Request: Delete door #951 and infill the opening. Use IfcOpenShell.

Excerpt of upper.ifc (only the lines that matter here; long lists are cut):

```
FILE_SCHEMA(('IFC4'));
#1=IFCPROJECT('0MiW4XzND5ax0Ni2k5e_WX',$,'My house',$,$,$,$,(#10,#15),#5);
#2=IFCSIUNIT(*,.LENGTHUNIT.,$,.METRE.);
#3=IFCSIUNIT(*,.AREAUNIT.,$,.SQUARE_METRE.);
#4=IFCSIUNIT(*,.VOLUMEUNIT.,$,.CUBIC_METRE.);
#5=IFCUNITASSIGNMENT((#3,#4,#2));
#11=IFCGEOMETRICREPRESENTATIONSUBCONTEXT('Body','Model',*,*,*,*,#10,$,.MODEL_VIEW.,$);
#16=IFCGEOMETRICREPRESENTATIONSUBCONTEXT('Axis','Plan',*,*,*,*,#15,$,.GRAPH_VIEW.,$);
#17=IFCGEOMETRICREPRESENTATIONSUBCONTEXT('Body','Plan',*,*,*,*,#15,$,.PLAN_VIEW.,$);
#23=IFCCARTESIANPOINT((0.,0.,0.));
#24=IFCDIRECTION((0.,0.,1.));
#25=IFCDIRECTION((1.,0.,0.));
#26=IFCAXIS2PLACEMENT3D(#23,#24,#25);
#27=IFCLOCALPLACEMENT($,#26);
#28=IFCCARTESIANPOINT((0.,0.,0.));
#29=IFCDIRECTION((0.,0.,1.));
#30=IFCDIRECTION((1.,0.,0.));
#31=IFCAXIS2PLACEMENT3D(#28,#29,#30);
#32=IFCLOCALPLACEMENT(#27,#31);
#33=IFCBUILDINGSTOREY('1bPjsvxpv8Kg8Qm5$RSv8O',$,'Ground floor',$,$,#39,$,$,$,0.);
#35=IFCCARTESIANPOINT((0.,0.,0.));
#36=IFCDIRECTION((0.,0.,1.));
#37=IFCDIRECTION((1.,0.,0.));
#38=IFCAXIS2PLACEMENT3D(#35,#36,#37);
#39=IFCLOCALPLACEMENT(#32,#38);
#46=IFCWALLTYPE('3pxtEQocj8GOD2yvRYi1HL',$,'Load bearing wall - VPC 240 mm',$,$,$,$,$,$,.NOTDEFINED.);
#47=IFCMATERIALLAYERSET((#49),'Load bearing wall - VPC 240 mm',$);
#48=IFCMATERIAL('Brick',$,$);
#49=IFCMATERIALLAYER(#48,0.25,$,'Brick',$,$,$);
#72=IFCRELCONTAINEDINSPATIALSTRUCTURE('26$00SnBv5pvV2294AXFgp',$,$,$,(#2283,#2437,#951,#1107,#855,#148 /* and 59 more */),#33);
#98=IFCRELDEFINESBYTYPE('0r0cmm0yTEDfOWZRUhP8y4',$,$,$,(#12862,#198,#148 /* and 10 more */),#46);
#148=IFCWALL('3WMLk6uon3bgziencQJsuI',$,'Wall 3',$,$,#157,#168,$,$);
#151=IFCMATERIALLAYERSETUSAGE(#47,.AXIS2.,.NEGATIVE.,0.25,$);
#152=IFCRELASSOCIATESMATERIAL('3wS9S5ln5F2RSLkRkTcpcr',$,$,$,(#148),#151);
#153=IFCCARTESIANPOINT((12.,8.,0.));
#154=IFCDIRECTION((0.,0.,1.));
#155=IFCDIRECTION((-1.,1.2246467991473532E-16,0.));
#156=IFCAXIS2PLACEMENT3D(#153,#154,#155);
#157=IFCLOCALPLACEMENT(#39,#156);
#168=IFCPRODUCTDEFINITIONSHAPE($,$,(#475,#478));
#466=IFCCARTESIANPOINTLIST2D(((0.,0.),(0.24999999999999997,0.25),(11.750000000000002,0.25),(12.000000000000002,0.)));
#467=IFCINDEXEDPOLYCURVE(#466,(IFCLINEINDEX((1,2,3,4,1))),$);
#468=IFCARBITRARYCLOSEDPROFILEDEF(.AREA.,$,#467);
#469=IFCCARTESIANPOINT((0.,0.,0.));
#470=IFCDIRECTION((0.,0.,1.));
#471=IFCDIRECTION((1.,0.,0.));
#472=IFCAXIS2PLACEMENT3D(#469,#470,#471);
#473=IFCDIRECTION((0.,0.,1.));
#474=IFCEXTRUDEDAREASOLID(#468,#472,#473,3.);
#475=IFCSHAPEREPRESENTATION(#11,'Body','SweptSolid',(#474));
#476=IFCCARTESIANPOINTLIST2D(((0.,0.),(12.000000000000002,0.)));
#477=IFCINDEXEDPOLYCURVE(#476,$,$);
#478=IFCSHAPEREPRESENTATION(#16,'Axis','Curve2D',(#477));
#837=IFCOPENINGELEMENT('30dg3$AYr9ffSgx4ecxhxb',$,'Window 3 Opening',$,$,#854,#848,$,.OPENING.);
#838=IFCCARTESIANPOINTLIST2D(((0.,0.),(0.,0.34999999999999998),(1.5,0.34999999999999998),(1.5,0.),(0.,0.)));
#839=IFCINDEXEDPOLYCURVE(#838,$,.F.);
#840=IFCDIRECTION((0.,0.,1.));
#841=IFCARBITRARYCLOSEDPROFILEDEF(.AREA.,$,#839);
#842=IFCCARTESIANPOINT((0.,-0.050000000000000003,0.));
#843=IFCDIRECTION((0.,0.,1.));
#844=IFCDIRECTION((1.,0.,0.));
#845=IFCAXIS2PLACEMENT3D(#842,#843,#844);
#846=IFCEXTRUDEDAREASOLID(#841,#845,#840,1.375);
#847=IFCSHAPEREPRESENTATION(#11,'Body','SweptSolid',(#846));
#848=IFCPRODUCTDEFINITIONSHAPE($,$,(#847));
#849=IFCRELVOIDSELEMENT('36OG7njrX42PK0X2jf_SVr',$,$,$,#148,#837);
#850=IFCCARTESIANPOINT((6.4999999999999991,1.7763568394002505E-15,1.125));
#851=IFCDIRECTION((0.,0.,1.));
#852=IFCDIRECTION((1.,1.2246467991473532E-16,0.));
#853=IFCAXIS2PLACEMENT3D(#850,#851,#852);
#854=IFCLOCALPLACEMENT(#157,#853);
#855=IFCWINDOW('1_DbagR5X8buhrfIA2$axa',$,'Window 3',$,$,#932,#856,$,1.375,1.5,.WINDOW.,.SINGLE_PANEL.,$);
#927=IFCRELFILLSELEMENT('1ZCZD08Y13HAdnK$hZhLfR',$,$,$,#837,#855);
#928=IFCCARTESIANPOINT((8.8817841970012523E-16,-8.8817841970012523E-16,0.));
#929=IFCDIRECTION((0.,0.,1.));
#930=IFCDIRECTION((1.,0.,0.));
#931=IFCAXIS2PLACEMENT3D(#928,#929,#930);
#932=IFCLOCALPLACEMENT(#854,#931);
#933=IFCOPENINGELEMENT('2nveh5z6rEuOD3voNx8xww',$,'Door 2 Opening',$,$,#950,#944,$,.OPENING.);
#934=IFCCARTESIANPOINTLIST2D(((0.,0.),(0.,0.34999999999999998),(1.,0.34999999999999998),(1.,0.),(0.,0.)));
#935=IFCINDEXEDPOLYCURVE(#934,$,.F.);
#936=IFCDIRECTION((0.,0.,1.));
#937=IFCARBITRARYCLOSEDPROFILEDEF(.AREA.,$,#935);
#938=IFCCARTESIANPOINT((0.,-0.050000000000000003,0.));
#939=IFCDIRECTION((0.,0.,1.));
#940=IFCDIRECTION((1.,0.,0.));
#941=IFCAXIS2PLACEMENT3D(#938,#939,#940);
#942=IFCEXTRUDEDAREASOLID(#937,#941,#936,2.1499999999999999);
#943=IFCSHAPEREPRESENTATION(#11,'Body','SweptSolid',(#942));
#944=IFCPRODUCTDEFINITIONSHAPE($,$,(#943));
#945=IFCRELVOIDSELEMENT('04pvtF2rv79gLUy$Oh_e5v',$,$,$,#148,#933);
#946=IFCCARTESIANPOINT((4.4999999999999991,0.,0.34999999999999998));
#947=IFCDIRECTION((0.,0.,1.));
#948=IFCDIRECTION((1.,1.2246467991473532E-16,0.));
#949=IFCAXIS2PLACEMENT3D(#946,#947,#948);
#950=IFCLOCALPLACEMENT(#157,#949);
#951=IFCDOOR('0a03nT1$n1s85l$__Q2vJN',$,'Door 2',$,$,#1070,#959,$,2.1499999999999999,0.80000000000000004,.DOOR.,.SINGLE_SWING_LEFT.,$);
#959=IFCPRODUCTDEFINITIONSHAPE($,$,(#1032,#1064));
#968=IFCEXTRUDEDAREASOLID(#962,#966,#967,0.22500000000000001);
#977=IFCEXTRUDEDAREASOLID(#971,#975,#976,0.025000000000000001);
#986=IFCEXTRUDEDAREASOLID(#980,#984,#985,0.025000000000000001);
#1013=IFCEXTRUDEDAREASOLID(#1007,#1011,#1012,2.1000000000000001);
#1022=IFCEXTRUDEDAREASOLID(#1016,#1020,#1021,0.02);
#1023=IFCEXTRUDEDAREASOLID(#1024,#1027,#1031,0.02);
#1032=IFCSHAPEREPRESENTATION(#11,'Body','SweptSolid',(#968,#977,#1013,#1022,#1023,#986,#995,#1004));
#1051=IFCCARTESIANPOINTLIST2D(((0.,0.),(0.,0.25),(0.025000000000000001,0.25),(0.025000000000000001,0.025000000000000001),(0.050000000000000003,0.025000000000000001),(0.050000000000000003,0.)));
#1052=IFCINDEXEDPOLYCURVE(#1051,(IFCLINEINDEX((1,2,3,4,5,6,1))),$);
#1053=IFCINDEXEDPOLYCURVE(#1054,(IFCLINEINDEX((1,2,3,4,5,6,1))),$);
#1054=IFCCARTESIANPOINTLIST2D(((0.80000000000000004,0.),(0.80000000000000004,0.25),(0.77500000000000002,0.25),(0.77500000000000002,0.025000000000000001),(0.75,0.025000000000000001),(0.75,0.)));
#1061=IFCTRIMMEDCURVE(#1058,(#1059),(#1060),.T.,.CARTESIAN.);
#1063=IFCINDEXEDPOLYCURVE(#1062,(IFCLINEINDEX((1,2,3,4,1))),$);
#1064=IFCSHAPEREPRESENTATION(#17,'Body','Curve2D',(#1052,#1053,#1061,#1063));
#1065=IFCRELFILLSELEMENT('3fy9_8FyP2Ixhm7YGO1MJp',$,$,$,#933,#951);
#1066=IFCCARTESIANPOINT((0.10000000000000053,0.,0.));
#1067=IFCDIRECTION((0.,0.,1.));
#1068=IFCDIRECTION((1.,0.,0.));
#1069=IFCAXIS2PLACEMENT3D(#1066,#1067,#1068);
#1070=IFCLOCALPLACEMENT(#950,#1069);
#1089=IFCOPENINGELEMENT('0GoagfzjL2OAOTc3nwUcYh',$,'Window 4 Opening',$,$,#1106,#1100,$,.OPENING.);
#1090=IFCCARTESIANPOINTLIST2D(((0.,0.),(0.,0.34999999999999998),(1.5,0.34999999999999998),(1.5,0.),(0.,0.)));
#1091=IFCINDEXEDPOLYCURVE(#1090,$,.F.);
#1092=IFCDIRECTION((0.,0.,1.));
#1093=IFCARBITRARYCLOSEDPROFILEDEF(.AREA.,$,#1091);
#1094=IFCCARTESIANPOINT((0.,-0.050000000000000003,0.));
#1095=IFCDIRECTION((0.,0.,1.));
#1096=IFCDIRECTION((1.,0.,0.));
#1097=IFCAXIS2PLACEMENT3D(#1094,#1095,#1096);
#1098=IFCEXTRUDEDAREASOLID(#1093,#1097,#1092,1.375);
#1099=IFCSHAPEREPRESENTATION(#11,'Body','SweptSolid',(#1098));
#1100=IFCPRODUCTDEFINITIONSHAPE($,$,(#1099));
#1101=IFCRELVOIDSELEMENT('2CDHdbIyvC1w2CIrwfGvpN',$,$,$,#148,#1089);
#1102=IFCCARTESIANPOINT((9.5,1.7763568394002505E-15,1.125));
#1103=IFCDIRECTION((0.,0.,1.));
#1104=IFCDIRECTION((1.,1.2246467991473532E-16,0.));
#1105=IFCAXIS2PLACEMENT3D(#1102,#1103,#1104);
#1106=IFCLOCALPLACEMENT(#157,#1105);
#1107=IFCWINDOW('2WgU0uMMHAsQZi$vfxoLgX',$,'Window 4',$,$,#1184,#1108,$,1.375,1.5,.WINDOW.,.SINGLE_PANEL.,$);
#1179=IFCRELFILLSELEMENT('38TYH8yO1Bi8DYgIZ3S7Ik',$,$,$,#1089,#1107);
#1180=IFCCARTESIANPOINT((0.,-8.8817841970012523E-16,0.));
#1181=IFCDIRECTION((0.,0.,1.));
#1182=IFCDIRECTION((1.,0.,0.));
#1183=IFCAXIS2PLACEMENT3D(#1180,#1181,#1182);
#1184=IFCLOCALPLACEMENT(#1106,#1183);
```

```python
import ifcopenshell
import ifcopenshell.api.feature
import ifcopenshell.api.root
import ifcopenshell.geom
import ifcopenshell.util.shape

model = ifcopenshell.open("upper.ifc")
settings = ifcopenshell.geom.settings()


def volume(element):
    """Net volume in cubic metres, openings subtracted."""
    shape = ifcopenshell.geom.create_shape(settings, element)
    return ifcopenshell.util.shape.get_volume(shape.geometry)


door = model.by_guid("0a03nT1$n1s85l$__Q2vJN")
opening = door.FillsVoids[0].RelatingOpeningElement
wall = opening.VoidsElements[0].RelatingBuildingElement
before = volume(wall)

ifcopenshell.api.root.remove_product(model, product=door)
ifcopenshell.api.feature.remove_feature(model, feature=opening)

after = volume(wall)

print(f"wall volume {before:.3f} -> {after:.3f} m3")

model.write("upper_updated.ifc")
```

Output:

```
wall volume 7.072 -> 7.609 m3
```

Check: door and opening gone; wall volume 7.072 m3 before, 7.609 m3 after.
